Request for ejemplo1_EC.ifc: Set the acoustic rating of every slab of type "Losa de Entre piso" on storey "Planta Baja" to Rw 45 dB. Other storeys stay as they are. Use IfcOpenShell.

First a look at what the model holds.

```python
import ifcopenshell
import ifcopenshell.util.element

model = ifcopenshell.open("ejemplo1_EC.ifc")
print(model.schema)
storey = next(s for s in model.by_type("IfcBuildingStorey") if s.Name == "Planta Baja")
slabs = [e for e in ifcopenshell.util.element.get_decomposition(storey) if e.is_a("IfcSlab")]
seen = {}
for e in slabs:
    element_type = ifcopenshell.util.element.get_type(e)
    key = (element_type.Name if element_type != e and element_type else None, ifcopenshell.util.element.get_pset(e, "Pset_SlabCommon", "AcousticRating"))
    seen[key] = seen.get(key, 0) + 1
for (name, value), count in sorted(seen.items(), key=str):
    print(count, "x", name, "|", value)
```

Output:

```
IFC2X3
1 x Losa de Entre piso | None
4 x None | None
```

```python
import ifcopenshell
import ifcopenshell.api.pset
import ifcopenshell.util.element

model = ifcopenshell.open("ejemplo1_EC.ifc")

storey = next(s for s in model.by_type("IfcBuildingStorey") if s.Name == "Planta Baja")
slabs = [e for e in ifcopenshell.util.element.get_decomposition(storey) if e.is_a("IfcSlab")]

count = 0
for e in slabs:
    element_type = ifcopenshell.util.element.get_type(e)
    if element_type in (None, e) or element_type.Name != "Losa de Entre piso":
        continue
    # add_pset returns the element's existing set when there is one.
    pset = ifcopenshell.api.pset.add_pset(model, product=e, name="Pset_SlabCommon")
    ifcopenshell.api.pset.edit_pset(model, pset=pset, properties={"AcousticRating": "Rw 45 dB"})
    count += 1

print(count, "slabs updated")

model.write("ejemplo1_EC-out.ifc")
```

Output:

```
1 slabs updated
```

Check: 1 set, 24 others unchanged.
